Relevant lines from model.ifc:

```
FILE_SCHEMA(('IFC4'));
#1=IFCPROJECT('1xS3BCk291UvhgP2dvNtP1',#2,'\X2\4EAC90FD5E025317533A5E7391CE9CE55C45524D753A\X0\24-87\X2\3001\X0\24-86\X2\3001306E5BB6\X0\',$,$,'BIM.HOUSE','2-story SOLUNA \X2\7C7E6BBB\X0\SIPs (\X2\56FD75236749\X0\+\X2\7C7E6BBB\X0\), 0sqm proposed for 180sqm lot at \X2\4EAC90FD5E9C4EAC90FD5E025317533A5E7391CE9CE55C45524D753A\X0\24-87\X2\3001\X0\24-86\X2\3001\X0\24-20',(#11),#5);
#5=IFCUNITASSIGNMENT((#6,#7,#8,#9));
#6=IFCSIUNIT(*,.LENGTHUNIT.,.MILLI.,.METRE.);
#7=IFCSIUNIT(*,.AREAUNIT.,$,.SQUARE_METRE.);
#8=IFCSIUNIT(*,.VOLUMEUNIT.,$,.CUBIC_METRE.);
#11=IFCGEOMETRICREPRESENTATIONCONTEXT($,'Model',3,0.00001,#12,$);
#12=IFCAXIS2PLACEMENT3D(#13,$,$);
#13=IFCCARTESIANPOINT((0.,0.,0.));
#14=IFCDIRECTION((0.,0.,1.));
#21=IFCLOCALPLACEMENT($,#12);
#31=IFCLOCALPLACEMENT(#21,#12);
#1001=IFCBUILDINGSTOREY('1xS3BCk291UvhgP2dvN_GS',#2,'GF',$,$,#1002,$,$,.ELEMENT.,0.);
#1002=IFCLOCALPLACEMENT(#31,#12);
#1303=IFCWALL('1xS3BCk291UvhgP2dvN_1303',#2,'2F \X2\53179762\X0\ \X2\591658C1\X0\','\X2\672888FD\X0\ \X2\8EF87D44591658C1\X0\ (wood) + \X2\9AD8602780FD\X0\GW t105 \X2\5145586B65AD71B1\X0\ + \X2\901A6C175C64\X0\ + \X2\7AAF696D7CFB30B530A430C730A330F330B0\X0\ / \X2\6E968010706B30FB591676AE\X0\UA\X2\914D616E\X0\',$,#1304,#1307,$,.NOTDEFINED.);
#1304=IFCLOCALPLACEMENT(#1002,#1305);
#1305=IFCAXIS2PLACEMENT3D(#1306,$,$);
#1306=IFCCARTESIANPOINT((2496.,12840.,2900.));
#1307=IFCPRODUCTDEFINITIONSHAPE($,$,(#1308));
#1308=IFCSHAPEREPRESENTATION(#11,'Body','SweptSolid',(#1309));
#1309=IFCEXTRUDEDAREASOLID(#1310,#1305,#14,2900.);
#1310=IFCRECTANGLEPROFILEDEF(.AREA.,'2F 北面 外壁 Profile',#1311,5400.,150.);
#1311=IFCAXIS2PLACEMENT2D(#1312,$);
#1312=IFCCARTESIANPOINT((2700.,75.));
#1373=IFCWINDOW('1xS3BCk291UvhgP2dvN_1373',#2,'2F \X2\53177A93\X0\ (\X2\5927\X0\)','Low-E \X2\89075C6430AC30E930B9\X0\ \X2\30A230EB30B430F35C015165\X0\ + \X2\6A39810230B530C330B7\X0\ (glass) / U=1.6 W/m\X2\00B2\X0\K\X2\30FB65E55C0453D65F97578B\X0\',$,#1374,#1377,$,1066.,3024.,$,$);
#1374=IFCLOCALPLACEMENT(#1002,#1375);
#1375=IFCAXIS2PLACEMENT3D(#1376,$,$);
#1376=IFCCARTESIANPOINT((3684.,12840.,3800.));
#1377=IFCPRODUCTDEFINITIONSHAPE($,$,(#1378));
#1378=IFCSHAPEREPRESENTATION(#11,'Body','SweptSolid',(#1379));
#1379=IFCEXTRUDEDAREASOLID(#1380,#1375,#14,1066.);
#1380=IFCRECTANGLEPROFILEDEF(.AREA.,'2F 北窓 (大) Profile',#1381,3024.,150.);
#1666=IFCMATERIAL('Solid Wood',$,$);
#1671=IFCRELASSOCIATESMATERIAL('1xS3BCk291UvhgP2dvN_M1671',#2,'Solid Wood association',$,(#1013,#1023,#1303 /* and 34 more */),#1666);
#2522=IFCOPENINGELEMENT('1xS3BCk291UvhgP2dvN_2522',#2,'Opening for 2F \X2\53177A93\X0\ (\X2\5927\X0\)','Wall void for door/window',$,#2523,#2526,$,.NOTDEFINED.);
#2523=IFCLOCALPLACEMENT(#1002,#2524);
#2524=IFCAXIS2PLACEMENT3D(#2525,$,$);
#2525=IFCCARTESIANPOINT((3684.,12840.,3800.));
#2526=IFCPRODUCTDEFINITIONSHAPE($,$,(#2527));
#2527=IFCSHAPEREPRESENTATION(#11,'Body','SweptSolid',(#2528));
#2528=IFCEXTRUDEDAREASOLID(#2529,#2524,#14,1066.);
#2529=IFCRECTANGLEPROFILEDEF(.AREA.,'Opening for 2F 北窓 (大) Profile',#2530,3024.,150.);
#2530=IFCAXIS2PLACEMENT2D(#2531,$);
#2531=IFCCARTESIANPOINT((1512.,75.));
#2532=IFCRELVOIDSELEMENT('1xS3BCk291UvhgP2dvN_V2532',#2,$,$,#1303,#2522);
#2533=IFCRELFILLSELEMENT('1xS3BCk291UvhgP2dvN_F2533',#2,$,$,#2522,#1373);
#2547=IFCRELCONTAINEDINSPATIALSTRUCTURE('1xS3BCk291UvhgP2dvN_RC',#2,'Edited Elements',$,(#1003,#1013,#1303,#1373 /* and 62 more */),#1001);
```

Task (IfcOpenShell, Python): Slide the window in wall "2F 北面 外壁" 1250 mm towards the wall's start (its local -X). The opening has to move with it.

```python
import ifcopenshell
import ifcopenshell.api.geometry
import ifcopenshell.util.placement
import ifcopenshell.util.unit

model = ifcopenshell.open("model.ifc")
unit_scale = ifcopenshell.util.unit.calculate_unit_scale(model)

window = model.by_id(1373)
opening = window.FillsVoids[0].RelatingOpeningElement
wall = opening.VoidsElements[0].RelatingBuildingElement

wall_matrix = ifcopenshell.util.placement.get_local_placement(wall.ObjectPlacement)
shift = wall_matrix[:3, 0] * -1.25 / unit_scale
before = ifcopenshell.util.placement.get_local_placement(window.ObjectPlacement)[:3, 3].copy()

# The window is not placed relative to its opening, so move both.
for product in (opening, window):
    matrix = ifcopenshell.util.placement.get_local_placement(product.ObjectPlacement)
    matrix[:3, 3] += shift
    ifcopenshell.api.geometry.edit_object_placement(model, product=product, matrix=matrix, is_si=False)

after = ifcopenshell.util.placement.get_local_placement(window.ObjectPlacement)[:3, 3]
print("window moved by", (after - before).round(3) + 0.0)

model.write("model_rev.ifc")
```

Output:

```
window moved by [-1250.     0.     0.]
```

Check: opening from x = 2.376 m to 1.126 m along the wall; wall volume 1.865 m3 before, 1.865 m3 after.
